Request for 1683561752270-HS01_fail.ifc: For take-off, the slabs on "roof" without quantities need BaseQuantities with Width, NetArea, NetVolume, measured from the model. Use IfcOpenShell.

First a look at what the model holds.

```python
import ifcopenshell
import ifcopenshell.util.element
import ifcopenshell.util.unit

model = ifcopenshell.open("1683561752270-HS01_fail.ifc")
print(model.schema)
for unit_type in ("LENGTHUNIT", "AREAUNIT", "VOLUMEUNIT"):
    print(unit_type, ifcopenshell.util.unit.calculate_unit_scale(model, unit_type))
storey = next(s for s in model.by_type("IfcBuildingStorey") if s.Name == "roof")
slabs = [e for e in ifcopenshell.util.element.get_decomposition(storey) if e.is_a("IfcSlab")]
for e in sorted(slabs, key=lambda e: e.id()):
    print(e.id(), e.is_a(), e.Name, list(ifcopenshell.util.element.get_psets(e, qtos_only=True)), sep=" | ")
```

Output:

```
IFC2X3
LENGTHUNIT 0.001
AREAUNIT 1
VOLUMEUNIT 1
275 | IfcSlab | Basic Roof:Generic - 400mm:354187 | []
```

```python
import ifcopenshell
import ifcopenshell.api.pset
import ifcopenshell.geom
import ifcopenshell.util.element
import ifcopenshell.util.shape
import ifcopenshell.util.unit

model = ifcopenshell.open("1683561752270-HS01_fail.ifc")
unit_scale = ifcopenshell.util.unit.calculate_unit_scale(model)
area_scale = ifcopenshell.util.unit.calculate_unit_scale(model, "AREAUNIT")
volume_scale = ifcopenshell.util.unit.calculate_unit_scale(model, "VOLUMEUNIT")
settings = ifcopenshell.geom.settings()

storey = next(s for s in model.by_type("IfcBuildingStorey") if s.Name == "roof")
slabs = [e for e in ifcopenshell.util.element.get_decomposition(storey) if e.is_a("IfcSlab")]

for e in sorted(slabs, key=lambda e: e.id()):
    if ifcopenshell.util.element.get_psets(e, qtos_only=True, should_inherit=False):
        continue
    # Geometry comes back in metres, in the element's own axes.
    shape = ifcopenshell.geom.create_shape(settings, e)
    values = {
        "Width": ifcopenshell.util.shape.get_z(shape.geometry) / unit_scale,
        "NetArea": ifcopenshell.util.shape.get_footprint_area(shape.geometry) / area_scale,
        "NetVolume": ifcopenshell.util.shape.get_volume(shape.geometry) / volume_scale,
    }
    qto = ifcopenshell.api.pset.add_qto(model, product=e, name="BaseQuantities")
    ifcopenshell.api.pset.edit_qto(model, qto=qto, properties=values)
    print(e.id(), {k: round(v, 3) for k, v in values.items()})

model.write("1683561752270-HS01_fail_edited.ifc")
```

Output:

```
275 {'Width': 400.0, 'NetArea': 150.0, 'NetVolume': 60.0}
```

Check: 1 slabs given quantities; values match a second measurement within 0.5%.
